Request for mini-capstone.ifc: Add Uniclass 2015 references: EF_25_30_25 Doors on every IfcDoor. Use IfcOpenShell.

First a look at what the model holds.

```python
import ifcopenshell

model = ifcopenshell.open("mini-capstone.ifc")
print(model.schema)
print("classifications:", [c.Name for c in model.by_type("IfcClassification")])
for ifc_class in ("IfcDoor", "IfcRoof", "IfcStair", "IfcWall", "IfcWindow"):
    print(ifc_class, len(model.by_type(ifc_class)))
```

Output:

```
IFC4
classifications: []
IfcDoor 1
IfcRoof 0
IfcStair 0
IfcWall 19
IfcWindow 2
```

```python
import ifcopenshell
import ifcopenshell.api.classification

model = ifcopenshell.open("mini-capstone.ifc")

system = ifcopenshell.api.classification.add_classification(model, classification="Uniclass 2015")

codes = {
    "IfcDoor": ("EF_25_30_25", "Doors"),
}
for ifc_class, (code, name) in codes.items():
    products = model.by_type(ifc_class)
    ifcopenshell.api.classification.add_reference(
        model, products=products, classification=system, identification=code, name=name
    )
    print(code, len(products))

model.write("mini-capstone_edited.ifc")
```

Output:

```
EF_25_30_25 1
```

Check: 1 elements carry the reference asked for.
